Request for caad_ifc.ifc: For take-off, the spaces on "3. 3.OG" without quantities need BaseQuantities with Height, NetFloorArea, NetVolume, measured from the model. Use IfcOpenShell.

First a look at what the model holds.

```python
import ifcopenshell
import ifcopenshell.util.element
import ifcopenshell.util.unit

model = ifcopenshell.open("caad_ifc.ifc")
print(model.schema)
for unit_type in ("LENGTHUNIT", "AREAUNIT", "VOLUMEUNIT"):
    print(unit_type, ifcopenshell.util.unit.calculate_unit_scale(model, unit_type))
storey = next(s for s in model.by_type("IfcBuildingStorey") if s.Name == "3. 3.OG")
spaces = [e for e in ifcopenshell.util.element.get_decomposition(storey) if e.is_a("IfcSpace")]
for e in sorted(spaces, key=lambda e: e.id()):
    print(e.id(), e.is_a(), e.Name, list(ifcopenshell.util.element.get_psets(e, qtos_only=True)), sep=" | ")
```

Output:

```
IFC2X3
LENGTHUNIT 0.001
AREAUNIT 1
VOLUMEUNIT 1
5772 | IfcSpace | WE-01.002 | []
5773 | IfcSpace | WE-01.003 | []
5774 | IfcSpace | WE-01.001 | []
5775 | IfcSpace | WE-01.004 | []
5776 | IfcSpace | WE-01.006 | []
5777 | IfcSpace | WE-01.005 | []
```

```python
import ifcopenshell
import ifcopenshell.api.pset
import ifcopenshell.geom
import ifcopenshell.util.element
import ifcopenshell.util.shape
import ifcopenshell.util.unit

model = ifcopenshell.open("caad_ifc.ifc")
unit_scale = ifcopenshell.util.unit.calculate_unit_scale(model)
area_scale = ifcopenshell.util.unit.calculate_unit_scale(model, "AREAUNIT")
volume_scale = ifcopenshell.util.unit.calculate_unit_scale(model, "VOLUMEUNIT")
settings = ifcopenshell.geom.settings()

storey = next(s for s in model.by_type("IfcBuildingStorey") if s.Name == "3. 3.OG")
spaces = [e for e in ifcopenshell.util.element.get_decomposition(storey) if e.is_a("IfcSpace")]

for e in sorted(spaces, key=lambda e: e.id()):
    if ifcopenshell.util.element.get_psets(e, qtos_only=True, should_inherit=False):
        continue
    # Geometry comes back in metres, in the element's own axes.
    shape = ifcopenshell.geom.create_shape(settings, e)
    values = {
        "Height": ifcopenshell.util.shape.get_z(shape.geometry) / unit_scale,
        "NetFloorArea": ifcopenshell.util.shape.get_footprint_area(shape.geometry) / area_scale,
        "NetVolume": ifcopenshell.util.shape.get_volume(shape.geometry) / volume_scale,
    }
    qto = ifcopenshell.api.pset.add_qto(model, product=e, name="BaseQuantities")
    ifcopenshell.api.pset.edit_qto(model, qto=qto, properties=values)
    print(e.id(), {k: round(v, 3) for k, v in values.items()})

model.write("caad_ifc_edited.ifc")
```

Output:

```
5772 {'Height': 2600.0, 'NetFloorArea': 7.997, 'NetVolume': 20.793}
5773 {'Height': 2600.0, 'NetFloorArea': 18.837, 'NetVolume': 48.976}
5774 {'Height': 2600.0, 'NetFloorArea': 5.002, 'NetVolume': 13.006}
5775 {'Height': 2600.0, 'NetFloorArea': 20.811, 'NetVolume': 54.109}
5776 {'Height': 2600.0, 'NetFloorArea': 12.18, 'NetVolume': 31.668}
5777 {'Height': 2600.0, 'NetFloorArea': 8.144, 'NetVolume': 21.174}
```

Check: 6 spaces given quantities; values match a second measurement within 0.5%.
